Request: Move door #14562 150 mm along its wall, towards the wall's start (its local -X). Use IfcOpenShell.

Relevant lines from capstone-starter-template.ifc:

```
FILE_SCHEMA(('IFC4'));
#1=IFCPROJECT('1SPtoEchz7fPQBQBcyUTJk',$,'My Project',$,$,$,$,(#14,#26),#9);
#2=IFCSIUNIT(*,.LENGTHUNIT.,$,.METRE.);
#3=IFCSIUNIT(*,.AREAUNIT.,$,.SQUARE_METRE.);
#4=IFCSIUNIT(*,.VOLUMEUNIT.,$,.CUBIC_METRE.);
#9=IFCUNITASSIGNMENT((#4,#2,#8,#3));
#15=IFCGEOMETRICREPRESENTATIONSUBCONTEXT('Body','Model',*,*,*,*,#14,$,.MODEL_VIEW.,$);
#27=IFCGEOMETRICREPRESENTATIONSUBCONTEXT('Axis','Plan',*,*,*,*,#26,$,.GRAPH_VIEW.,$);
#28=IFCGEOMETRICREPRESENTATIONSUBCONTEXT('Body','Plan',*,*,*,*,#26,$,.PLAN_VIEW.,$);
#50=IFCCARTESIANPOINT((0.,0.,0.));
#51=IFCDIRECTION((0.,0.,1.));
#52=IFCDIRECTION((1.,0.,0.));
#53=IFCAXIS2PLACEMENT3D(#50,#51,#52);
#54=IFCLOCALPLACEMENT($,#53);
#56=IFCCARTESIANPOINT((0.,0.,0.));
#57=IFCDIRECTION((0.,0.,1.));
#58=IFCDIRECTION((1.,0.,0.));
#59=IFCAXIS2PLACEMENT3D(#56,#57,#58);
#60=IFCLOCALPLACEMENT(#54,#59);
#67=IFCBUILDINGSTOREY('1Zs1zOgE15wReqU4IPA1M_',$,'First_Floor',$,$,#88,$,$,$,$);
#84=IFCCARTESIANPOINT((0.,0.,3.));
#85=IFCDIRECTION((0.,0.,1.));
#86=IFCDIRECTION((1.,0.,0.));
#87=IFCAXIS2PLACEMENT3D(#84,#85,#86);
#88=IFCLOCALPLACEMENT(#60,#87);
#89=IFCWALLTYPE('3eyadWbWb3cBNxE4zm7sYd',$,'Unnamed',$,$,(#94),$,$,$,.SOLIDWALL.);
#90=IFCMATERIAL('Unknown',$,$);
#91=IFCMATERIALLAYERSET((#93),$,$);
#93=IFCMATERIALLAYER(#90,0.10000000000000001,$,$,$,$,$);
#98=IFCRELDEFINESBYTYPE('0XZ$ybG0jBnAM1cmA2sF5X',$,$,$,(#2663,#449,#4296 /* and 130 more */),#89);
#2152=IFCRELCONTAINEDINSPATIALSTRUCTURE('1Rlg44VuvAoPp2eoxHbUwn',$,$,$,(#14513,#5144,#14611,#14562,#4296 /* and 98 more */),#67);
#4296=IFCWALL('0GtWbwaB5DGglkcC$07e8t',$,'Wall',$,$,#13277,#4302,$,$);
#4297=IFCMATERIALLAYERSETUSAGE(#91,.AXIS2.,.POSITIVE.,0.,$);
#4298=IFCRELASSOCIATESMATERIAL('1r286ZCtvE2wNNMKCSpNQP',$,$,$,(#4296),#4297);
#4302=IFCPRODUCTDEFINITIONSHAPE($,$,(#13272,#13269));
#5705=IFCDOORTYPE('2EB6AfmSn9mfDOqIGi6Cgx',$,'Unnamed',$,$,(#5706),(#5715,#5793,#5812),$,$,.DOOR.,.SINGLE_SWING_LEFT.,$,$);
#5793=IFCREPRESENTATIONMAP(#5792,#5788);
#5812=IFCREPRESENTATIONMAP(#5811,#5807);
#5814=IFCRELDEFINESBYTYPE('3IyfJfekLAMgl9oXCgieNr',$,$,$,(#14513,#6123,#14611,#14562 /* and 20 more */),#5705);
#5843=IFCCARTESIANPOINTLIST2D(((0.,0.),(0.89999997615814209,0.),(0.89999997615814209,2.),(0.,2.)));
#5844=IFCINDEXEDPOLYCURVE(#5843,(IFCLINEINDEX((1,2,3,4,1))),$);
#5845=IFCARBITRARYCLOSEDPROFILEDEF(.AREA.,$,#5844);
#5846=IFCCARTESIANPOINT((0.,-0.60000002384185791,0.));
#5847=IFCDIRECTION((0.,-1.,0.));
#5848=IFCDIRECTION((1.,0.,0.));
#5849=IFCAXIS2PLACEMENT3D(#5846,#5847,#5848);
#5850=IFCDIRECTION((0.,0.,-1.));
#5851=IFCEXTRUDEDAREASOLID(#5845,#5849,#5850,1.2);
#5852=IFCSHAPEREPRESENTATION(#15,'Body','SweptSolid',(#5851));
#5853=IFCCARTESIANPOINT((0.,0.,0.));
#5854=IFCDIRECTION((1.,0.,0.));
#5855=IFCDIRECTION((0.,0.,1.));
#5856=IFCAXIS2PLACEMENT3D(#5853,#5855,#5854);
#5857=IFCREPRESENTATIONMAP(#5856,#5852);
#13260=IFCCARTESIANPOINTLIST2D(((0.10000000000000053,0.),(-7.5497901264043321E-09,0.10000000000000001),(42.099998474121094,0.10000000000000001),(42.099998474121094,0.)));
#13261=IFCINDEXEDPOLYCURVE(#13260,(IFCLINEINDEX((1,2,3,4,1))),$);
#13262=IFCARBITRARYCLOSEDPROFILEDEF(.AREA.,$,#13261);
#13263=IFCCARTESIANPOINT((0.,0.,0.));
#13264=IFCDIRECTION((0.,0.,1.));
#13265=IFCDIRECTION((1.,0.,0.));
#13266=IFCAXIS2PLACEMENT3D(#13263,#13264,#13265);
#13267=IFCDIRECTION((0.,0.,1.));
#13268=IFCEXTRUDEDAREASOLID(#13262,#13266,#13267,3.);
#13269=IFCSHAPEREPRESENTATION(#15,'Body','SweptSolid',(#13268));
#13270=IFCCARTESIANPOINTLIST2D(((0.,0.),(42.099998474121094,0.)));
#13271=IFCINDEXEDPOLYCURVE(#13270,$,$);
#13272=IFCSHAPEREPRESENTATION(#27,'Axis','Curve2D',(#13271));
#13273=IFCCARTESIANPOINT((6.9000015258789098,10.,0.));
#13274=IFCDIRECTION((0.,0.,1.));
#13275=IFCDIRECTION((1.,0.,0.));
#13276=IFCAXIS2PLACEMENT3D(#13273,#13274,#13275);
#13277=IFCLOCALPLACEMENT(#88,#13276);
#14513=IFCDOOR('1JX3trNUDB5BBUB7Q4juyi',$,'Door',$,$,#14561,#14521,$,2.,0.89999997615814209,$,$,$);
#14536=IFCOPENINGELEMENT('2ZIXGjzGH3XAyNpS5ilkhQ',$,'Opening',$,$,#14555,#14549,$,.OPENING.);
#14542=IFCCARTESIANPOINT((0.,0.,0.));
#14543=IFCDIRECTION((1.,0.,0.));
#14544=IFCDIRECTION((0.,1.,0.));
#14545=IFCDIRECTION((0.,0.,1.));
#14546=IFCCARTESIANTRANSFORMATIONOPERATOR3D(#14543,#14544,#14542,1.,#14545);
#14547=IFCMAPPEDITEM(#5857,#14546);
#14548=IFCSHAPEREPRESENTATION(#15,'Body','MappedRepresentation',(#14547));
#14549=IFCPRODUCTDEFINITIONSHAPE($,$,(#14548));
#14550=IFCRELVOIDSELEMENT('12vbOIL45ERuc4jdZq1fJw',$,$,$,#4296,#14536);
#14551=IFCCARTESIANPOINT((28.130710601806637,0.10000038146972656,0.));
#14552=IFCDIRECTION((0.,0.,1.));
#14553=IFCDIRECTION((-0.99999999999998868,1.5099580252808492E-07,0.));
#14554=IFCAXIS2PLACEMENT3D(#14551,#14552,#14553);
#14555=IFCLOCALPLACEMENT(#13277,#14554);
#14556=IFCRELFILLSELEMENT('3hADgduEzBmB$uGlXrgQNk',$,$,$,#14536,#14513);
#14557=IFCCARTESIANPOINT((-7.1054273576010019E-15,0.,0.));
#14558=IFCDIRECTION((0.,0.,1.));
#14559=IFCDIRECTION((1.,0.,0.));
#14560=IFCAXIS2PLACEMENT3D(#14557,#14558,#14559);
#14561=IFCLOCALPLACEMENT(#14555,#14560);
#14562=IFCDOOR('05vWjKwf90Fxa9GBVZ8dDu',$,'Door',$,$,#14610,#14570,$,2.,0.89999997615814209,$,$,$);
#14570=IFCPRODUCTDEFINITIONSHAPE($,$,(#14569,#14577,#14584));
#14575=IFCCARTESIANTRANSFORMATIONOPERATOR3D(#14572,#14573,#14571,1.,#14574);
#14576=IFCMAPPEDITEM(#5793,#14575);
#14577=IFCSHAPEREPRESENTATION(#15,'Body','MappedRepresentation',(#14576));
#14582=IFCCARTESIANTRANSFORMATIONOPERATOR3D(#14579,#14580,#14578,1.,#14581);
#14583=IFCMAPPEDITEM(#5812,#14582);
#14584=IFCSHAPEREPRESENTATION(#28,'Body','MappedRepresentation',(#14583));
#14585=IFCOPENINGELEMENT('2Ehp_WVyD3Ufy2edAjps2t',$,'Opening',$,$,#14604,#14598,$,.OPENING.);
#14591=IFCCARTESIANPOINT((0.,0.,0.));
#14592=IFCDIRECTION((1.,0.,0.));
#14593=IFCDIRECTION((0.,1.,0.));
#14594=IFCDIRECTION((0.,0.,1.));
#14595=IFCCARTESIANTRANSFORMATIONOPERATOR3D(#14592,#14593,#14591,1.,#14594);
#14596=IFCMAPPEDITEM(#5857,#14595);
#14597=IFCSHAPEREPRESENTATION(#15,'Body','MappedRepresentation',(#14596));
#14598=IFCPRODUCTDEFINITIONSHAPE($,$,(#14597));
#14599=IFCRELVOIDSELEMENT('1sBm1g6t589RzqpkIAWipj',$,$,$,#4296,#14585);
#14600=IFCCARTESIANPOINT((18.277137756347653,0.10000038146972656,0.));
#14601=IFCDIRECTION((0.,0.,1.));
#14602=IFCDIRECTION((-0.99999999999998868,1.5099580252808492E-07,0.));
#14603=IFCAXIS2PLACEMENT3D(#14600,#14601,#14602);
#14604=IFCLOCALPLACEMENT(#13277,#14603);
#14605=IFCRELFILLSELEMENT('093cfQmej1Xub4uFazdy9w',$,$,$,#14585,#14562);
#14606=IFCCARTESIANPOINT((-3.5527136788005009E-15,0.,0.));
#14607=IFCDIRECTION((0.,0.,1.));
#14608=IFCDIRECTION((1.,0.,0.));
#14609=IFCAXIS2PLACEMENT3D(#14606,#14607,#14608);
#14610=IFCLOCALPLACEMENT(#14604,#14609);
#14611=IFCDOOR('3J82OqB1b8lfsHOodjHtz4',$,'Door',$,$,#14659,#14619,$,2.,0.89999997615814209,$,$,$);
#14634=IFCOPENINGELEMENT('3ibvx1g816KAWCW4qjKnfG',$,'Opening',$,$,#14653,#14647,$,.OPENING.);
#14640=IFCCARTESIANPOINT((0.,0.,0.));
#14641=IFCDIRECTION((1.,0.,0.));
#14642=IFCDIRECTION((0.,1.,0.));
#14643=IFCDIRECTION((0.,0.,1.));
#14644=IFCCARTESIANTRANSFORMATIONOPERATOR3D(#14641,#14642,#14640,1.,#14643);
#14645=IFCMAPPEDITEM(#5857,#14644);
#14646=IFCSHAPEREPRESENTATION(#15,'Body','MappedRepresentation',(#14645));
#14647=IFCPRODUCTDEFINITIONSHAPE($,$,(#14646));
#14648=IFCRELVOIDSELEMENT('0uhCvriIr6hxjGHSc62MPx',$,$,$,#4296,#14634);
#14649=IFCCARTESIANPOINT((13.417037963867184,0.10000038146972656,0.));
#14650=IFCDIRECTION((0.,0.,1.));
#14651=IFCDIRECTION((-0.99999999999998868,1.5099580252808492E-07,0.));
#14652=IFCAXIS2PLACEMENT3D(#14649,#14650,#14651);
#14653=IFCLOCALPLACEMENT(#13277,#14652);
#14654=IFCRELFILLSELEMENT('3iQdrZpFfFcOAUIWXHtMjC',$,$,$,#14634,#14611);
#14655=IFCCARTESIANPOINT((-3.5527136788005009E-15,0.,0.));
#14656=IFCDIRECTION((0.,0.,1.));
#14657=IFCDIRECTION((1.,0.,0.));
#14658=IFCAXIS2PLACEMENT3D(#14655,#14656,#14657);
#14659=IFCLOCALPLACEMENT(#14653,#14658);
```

```python
import ifcopenshell
import ifcopenshell.api.geometry
import ifcopenshell.util.placement
import ifcopenshell.util.unit

model = ifcopenshell.open("capstone-starter-template.ifc")
unit_scale = ifcopenshell.util.unit.calculate_unit_scale(model)

door = model.by_guid("05vWjKwf90Fxa9GBVZ8dDu")
opening = door.FillsVoids[0].RelatingOpeningElement
wall = opening.VoidsElements[0].RelatingBuildingElement

wall_matrix = ifcopenshell.util.placement.get_local_placement(wall.ObjectPlacement)
shift = wall_matrix[:3, 0] * -0.15 / unit_scale
before = ifcopenshell.util.placement.get_local_placement(door.ObjectPlacement)[:3, 3].copy()

# The door is placed relative to its opening, so it follows when the opening moves.
matrix = ifcopenshell.util.placement.get_local_placement(opening.ObjectPlacement)
matrix[:3, 3] += shift
ifcopenshell.api.geometry.edit_object_placement(
    model, product=opening, matrix=matrix, is_si=False, should_transform_children=True
)

after = ifcopenshell.util.placement.get_local_placement(door.ObjectPlacement)[:3, 3]
print("door moved by", (after - before).round(3) + 0.0)

model.write("capstone-starter-template_edited.ifc")
```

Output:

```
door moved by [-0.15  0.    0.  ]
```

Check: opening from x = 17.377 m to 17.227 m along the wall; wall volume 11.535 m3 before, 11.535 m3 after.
